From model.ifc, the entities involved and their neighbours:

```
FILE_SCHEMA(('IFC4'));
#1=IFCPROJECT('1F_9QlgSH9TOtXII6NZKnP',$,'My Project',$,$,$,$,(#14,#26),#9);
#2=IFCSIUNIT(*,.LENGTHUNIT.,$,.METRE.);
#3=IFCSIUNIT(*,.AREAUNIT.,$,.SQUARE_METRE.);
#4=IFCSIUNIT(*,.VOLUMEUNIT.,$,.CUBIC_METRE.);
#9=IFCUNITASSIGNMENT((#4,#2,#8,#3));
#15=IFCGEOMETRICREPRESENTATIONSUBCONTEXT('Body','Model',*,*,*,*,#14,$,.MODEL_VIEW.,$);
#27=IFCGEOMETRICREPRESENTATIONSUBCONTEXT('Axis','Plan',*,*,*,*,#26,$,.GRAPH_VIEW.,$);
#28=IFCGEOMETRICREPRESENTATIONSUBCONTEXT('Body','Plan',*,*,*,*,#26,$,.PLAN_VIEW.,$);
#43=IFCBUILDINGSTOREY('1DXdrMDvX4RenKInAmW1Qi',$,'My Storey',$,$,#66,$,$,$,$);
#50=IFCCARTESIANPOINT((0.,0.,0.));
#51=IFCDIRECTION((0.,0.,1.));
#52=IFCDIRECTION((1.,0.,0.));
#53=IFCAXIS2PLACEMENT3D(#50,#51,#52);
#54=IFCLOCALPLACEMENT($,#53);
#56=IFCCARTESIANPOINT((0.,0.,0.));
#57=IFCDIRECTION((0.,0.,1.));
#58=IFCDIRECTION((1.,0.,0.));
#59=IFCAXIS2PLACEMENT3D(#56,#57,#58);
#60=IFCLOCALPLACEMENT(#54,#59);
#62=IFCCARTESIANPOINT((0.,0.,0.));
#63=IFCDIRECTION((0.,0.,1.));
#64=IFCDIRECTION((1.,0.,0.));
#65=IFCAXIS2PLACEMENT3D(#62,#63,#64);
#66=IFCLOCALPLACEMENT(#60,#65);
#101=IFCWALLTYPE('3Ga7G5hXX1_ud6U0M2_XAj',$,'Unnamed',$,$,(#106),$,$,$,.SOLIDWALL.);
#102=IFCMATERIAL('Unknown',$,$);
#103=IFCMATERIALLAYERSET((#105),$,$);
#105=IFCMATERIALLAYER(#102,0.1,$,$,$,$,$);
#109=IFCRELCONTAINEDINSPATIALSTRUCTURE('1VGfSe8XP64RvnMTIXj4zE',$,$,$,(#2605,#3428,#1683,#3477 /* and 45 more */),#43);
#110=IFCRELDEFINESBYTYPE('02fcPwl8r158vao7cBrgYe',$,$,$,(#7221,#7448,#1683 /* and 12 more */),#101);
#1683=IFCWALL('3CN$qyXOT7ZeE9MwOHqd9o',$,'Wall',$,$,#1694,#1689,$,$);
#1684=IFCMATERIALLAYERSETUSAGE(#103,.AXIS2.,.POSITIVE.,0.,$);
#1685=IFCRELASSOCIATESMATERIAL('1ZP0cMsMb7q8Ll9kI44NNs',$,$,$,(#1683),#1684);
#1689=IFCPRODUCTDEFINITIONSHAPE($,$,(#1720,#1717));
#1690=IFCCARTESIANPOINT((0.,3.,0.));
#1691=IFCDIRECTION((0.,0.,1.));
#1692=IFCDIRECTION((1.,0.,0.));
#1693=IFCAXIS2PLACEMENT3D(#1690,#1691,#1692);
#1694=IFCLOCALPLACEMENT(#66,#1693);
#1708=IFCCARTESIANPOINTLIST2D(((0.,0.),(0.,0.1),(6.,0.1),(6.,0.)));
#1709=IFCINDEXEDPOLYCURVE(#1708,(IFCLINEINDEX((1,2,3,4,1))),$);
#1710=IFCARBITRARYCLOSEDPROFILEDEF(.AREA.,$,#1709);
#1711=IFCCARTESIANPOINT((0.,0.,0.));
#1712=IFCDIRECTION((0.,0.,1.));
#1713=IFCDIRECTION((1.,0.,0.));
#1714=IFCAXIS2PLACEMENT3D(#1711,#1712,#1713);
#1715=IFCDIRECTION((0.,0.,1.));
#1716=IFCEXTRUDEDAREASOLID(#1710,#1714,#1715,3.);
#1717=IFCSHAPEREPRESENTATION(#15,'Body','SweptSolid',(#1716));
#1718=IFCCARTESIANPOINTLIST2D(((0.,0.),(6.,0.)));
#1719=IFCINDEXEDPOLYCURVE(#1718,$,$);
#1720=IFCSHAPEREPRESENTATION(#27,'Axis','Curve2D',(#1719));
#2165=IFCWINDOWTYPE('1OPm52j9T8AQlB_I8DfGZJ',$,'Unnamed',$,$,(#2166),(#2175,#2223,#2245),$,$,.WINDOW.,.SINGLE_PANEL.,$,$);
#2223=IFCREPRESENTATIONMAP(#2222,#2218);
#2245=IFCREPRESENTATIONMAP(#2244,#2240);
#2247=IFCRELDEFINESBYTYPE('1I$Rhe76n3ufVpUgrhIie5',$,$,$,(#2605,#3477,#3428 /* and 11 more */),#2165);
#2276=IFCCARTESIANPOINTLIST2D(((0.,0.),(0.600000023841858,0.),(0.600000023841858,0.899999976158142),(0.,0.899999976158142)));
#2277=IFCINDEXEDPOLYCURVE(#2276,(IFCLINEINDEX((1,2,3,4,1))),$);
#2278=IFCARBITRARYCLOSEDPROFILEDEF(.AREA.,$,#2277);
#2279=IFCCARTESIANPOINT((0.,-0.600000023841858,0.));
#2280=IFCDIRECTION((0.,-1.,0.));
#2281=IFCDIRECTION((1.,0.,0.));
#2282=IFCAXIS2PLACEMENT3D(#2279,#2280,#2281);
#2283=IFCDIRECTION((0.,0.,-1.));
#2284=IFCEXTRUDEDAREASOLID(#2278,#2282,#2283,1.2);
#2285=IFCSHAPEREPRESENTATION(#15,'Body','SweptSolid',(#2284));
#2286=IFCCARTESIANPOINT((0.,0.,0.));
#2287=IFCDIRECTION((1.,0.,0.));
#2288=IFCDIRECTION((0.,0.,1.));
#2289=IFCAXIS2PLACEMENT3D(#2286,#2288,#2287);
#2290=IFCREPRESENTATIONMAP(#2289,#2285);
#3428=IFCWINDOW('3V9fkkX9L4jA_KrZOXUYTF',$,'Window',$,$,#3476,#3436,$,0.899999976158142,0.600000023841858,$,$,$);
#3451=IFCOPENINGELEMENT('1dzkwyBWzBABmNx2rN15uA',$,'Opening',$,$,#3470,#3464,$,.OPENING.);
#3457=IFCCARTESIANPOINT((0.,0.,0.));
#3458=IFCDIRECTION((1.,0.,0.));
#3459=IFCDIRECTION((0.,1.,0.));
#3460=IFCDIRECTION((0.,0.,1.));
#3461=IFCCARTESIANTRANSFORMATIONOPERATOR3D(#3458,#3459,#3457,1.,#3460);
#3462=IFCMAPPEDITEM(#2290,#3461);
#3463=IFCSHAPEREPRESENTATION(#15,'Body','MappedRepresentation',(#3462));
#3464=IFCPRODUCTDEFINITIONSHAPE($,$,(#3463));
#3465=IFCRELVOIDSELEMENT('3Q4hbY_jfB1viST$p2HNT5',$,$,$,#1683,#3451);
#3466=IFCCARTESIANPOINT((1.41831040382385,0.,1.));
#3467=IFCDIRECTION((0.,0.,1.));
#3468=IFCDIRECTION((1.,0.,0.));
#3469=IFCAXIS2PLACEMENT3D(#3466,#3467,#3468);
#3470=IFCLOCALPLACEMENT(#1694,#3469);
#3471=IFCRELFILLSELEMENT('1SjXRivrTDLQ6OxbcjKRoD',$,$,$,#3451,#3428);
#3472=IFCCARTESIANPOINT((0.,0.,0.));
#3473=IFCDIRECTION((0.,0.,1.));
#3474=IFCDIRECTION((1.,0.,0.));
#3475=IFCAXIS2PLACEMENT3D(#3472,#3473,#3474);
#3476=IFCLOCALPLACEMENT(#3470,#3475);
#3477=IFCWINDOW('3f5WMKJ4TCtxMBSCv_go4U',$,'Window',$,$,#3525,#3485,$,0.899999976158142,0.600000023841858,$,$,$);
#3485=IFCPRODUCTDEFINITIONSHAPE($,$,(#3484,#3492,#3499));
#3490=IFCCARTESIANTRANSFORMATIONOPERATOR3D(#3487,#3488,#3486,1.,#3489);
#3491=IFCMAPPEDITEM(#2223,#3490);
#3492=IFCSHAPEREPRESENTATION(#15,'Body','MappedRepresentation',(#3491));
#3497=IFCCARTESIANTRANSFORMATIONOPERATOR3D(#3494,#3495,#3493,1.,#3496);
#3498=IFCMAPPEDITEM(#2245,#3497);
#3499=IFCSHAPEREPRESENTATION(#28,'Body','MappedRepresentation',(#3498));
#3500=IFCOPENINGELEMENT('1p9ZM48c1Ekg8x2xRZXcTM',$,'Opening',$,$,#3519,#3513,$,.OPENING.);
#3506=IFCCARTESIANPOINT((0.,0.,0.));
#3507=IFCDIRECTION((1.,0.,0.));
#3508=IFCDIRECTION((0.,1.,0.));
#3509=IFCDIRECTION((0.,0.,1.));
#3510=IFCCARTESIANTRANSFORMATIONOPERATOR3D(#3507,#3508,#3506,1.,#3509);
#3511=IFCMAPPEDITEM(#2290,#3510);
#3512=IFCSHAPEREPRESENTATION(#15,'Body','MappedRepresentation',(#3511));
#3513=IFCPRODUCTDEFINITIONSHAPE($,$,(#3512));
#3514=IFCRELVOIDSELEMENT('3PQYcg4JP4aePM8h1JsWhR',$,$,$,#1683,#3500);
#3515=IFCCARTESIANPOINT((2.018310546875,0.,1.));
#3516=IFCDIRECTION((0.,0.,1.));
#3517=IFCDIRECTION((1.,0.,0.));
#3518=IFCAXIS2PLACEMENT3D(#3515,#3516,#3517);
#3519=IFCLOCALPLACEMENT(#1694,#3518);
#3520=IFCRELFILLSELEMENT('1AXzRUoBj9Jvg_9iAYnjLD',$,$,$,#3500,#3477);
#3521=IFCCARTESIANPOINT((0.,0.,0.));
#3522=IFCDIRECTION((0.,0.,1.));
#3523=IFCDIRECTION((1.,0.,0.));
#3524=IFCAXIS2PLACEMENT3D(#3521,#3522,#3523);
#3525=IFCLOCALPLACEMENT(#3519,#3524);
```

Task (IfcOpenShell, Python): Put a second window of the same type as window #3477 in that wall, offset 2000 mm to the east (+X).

```python
import ifcopenshell
import ifcopenshell.api.feature
import ifcopenshell.api.geometry
import ifcopenshell.api.root
import ifcopenshell.geom
import ifcopenshell.util.element
import ifcopenshell.util.placement
import ifcopenshell.util.shape
import ifcopenshell.util.unit

model = ifcopenshell.open("model.ifc")
unit_scale = ifcopenshell.util.unit.calculate_unit_scale(model)
settings = ifcopenshell.geom.settings()


def volume(element):
    """Net volume in cubic metres, openings subtracted."""
    shape = ifcopenshell.geom.create_shape(settings, element)
    return ifcopenshell.util.shape.get_volume(shape.geometry)


window = model.by_id(3477)
opening = window.FillsVoids[0].RelatingOpeningElement
wall = opening.VoidsElements[0].RelatingBuildingElement
before = volume(wall)
shift = ifcopenshell.util.placement.get_local_placement(wall.ObjectPlacement)[:3, 0] * 2 / unit_scale

# copy_class copies the void relationship, type, container and properties, but no geometry.
new_opening = ifcopenshell.api.root.copy_class(model, product=opening)
new_opening.Representation = ifcopenshell.util.element.copy_deep(
    model, opening.Representation, exclude=["IfcGeometricRepresentationContext", "IfcRepresentationMap"]
)
new_window = ifcopenshell.api.root.copy_class(model, product=window)
new_window.Representation = ifcopenshell.util.element.copy_deep(
    model, window.Representation, exclude=["IfcGeometricRepresentationContext", "IfcRepresentationMap"]
)
ifcopenshell.api.feature.add_filling(model, opening=new_opening, element=new_window)

for old, new in ((opening, new_opening), (window, new_window)):
    matrix = ifcopenshell.util.placement.get_local_placement(old.ObjectPlacement)
    matrix[:3, 3] += shift
    ifcopenshell.api.geometry.edit_object_placement(model, product=new, matrix=matrix, is_si=False)

after = volume(wall)

print(f"wall volume {before:.3f} -> {after:.3f} m3")

model.write("model_rev.ifc")
```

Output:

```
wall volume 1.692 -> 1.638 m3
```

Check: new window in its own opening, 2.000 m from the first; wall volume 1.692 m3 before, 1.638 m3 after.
